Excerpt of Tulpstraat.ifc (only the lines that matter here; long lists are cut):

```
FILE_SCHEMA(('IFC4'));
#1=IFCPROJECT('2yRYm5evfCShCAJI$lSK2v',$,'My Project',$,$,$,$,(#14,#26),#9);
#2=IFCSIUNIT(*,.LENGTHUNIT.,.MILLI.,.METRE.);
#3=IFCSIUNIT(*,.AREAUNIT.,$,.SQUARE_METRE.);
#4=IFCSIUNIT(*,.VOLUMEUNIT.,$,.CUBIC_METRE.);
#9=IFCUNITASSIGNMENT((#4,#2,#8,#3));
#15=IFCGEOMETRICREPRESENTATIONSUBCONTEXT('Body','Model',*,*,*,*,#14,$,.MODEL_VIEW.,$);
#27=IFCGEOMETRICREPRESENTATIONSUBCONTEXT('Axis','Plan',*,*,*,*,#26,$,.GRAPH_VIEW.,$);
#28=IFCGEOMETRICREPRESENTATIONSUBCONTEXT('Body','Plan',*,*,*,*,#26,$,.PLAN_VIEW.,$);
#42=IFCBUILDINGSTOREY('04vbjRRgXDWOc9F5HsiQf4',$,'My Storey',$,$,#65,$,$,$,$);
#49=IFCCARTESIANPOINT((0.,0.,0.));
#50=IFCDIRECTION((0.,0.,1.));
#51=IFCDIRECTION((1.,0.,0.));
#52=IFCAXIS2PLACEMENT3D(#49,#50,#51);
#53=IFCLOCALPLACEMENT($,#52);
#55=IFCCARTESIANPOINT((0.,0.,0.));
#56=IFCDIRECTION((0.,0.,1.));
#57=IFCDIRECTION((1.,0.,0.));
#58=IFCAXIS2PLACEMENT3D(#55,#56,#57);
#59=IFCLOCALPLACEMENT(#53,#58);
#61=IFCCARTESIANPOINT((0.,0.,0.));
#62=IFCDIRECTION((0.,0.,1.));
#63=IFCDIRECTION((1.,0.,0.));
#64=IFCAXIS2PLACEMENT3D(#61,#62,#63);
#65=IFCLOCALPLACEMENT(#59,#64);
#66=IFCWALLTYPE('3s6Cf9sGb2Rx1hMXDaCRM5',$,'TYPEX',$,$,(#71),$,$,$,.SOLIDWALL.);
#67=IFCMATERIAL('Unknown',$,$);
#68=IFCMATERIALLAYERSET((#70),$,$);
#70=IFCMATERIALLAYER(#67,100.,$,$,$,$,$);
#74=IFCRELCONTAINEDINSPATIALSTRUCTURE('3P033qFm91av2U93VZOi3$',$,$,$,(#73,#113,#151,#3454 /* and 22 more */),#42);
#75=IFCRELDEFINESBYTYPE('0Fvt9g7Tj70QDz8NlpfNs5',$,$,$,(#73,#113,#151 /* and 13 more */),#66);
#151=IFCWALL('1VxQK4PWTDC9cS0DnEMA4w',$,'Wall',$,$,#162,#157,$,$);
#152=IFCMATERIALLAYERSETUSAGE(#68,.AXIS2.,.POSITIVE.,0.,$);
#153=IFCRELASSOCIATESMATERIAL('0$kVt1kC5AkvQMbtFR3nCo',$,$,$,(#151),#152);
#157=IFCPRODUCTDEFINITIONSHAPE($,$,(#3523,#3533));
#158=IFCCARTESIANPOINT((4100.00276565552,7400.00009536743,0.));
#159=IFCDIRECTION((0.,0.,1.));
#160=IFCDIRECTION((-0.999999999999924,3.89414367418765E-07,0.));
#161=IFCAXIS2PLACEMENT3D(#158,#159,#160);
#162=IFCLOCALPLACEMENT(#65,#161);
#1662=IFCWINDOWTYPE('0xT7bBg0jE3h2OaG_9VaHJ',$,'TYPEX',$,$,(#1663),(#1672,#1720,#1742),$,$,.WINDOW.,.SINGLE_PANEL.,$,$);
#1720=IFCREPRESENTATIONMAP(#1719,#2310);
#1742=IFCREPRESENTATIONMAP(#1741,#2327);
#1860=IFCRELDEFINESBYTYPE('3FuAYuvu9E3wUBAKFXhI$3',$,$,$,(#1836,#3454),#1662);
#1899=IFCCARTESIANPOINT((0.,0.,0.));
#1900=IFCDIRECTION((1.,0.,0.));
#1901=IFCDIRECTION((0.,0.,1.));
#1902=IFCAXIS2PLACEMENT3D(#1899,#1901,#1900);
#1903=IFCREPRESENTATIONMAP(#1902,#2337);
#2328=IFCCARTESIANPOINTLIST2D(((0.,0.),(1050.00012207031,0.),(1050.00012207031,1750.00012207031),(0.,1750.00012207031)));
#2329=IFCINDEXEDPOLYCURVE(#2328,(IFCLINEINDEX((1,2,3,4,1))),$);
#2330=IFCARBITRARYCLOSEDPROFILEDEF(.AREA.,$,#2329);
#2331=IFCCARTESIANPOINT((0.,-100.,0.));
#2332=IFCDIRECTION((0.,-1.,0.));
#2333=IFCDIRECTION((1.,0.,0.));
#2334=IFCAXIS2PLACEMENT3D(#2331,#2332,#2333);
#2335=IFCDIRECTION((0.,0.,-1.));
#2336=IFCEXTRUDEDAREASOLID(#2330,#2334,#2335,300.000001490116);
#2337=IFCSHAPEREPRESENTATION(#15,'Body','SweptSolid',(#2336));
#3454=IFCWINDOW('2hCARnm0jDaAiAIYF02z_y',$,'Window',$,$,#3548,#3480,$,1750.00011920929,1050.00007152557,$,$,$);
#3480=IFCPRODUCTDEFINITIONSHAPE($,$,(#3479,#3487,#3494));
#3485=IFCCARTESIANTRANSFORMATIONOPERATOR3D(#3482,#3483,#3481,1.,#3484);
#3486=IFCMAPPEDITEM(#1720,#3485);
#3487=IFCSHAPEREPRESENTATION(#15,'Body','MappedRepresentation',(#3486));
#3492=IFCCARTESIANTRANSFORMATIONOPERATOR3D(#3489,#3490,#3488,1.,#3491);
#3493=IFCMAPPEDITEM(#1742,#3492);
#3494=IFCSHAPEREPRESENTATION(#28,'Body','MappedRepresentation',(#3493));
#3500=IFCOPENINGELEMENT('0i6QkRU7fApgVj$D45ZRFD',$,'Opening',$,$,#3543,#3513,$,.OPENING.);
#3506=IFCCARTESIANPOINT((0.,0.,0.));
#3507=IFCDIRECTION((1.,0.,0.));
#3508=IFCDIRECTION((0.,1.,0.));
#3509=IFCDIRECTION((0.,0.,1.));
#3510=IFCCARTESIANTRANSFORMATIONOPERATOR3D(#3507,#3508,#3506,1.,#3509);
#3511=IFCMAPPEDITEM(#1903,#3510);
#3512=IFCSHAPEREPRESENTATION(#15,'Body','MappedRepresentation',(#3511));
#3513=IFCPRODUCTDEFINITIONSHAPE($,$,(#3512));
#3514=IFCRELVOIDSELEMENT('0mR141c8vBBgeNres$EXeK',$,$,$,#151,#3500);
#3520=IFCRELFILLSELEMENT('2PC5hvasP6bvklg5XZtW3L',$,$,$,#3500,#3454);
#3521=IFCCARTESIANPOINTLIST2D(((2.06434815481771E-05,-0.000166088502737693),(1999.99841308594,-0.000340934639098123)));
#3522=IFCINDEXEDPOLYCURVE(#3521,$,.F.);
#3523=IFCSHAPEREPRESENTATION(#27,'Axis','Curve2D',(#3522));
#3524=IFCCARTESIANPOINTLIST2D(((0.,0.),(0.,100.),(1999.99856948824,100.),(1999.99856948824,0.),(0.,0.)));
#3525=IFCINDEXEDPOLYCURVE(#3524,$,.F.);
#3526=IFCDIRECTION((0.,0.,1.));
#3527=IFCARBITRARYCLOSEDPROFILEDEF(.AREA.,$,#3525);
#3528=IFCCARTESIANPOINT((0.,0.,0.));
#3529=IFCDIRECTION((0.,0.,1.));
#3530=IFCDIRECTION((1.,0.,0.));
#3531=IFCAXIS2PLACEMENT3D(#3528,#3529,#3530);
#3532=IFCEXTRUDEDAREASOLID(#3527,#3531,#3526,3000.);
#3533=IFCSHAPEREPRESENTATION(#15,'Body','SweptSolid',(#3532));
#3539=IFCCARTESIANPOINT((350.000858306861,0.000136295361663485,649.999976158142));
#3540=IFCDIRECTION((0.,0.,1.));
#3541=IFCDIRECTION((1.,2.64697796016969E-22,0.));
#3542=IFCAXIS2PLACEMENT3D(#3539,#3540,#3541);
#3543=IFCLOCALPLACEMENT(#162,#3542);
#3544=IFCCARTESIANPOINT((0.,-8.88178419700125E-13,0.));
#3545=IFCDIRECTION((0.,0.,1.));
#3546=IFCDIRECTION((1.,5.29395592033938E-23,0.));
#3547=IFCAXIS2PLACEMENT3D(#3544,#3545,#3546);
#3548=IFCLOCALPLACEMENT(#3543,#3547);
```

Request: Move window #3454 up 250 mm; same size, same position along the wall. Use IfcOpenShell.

```python
import numpy as np
import ifcopenshell
import ifcopenshell.api.geometry
import ifcopenshell.util.placement
import ifcopenshell.util.unit

model = ifcopenshell.open("Tulpstraat.ifc")
unit_scale = ifcopenshell.util.unit.calculate_unit_scale(model)

window = model.by_guid("2hCARnm0jDaAiAIYF02z_y")
opening = window.FillsVoids[0].RelatingOpeningElement
dz = 0.25 / unit_scale

shift = np.array([0.0, 0.0, dz])
# The window is placed relative to its opening, so it follows when the opening moves.
matrix = ifcopenshell.util.placement.get_local_placement(opening.ObjectPlacement)
matrix[:3, 3] += shift
ifcopenshell.api.geometry.edit_object_placement(
    model, product=opening, matrix=matrix, is_si=False, should_transform_children=True
)

print(f"moved by {dz * unit_scale:+.3f} m")

model.write("Tulpstraat-out.ifc")
```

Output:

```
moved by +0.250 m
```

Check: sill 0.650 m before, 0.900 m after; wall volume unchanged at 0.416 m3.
